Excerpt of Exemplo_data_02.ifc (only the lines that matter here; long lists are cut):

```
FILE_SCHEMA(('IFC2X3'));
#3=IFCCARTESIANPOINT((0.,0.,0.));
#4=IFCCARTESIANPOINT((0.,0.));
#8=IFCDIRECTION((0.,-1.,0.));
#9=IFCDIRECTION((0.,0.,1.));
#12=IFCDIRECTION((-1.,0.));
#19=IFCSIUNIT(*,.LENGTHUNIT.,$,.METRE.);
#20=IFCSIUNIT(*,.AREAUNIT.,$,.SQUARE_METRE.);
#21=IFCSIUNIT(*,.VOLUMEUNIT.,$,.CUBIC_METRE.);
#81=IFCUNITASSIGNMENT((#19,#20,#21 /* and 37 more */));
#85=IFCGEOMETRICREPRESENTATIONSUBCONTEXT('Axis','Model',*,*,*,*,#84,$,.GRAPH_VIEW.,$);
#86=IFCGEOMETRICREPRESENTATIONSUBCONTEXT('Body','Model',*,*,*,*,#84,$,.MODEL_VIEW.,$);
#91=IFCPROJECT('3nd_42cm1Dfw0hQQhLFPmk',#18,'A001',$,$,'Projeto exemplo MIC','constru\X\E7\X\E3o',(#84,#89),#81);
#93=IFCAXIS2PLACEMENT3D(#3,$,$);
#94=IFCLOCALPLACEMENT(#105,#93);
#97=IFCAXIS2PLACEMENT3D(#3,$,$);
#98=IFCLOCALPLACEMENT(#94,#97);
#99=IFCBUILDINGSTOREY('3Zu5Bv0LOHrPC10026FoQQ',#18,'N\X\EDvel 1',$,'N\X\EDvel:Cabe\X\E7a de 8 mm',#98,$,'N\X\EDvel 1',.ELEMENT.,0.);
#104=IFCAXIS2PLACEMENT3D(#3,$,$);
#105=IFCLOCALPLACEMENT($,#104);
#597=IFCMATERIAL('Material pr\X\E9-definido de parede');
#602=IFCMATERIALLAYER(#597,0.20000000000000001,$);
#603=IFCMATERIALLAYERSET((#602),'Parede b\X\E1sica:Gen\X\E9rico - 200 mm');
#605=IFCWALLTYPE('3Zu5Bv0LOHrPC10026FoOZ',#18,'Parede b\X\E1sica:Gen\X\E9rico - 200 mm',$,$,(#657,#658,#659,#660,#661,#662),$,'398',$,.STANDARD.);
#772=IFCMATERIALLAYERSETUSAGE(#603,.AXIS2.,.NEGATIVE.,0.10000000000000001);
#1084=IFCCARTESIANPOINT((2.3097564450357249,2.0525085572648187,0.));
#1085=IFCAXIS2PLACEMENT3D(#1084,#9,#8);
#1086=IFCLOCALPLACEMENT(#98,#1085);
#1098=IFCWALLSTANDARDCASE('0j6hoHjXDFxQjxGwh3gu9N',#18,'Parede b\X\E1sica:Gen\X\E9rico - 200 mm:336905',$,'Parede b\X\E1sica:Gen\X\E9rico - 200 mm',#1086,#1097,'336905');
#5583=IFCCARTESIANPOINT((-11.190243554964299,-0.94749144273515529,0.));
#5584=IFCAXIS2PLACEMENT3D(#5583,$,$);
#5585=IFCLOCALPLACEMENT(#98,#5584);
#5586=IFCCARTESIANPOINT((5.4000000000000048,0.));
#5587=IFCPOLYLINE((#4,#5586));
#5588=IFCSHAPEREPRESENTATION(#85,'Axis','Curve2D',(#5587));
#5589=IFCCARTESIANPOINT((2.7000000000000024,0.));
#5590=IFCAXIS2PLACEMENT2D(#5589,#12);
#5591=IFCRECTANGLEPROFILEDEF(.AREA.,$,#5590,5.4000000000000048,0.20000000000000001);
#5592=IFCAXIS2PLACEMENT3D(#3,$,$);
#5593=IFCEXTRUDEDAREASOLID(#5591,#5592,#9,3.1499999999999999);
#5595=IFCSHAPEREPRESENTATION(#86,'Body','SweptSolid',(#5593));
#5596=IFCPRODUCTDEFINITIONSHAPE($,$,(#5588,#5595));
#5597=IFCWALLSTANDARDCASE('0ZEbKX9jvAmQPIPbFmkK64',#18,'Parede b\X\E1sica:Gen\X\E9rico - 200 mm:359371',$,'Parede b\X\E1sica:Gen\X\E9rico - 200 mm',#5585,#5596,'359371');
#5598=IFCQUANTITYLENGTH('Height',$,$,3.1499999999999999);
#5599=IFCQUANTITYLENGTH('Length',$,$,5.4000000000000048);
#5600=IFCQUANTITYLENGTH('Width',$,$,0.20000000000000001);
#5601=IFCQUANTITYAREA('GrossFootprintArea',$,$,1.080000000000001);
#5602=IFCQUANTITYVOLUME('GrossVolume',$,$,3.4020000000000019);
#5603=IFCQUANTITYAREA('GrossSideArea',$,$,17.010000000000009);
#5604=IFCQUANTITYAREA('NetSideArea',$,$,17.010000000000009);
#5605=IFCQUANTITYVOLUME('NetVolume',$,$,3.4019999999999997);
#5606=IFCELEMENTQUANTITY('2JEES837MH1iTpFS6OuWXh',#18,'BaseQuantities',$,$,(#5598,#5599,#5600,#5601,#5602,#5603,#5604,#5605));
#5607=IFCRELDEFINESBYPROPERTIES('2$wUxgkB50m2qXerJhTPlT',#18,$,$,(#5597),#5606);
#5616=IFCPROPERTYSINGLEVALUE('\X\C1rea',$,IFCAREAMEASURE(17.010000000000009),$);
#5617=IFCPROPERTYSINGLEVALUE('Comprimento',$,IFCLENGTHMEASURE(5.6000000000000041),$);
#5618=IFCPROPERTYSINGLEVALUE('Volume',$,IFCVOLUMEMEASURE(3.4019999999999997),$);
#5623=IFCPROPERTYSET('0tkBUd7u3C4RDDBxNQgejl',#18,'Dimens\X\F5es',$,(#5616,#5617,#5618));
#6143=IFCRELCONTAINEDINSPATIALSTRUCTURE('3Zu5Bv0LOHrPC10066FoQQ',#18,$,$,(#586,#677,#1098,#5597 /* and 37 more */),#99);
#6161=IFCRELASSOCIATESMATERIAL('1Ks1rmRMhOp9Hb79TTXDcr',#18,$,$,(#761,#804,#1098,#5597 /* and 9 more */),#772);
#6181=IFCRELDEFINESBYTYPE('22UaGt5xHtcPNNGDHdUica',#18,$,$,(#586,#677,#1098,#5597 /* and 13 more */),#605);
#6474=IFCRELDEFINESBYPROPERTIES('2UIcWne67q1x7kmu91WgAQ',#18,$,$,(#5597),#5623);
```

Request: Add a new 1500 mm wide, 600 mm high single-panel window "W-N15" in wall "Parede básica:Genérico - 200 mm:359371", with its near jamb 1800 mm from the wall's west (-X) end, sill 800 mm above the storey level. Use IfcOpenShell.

```python
import numpy as np
import ifcopenshell
import ifcopenshell.api.feature
import ifcopenshell.api.geometry
import ifcopenshell.api.pset
import ifcopenshell.api.root
import ifcopenshell.api.spatial
import ifcopenshell.api.type
import ifcopenshell.geom
import ifcopenshell.util.element
import ifcopenshell.util.placement
import ifcopenshell.util.representation
import ifcopenshell.util.shape
import ifcopenshell.util.unit

model = ifcopenshell.open("Exemplo_data_02.ifc")
unit_scale = ifcopenshell.util.unit.calculate_unit_scale(model)
area_scale = ifcopenshell.util.unit.calculate_unit_scale(model, "AREAUNIT")
volume_scale = ifcopenshell.util.unit.calculate_unit_scale(model, "VOLUMEUNIT")
settings = ifcopenshell.geom.settings()


def volume(element):
    """Net volume in cubic metres, openings subtracted."""
    shape = ifcopenshell.geom.create_shape(settings, element)
    return ifcopenshell.util.shape.get_volume(shape.geometry)


wall = model.by_guid("0ZEbKX9jvAmQPIPbFmkK64")
storey = ifcopenshell.util.element.get_container(wall, ifc_class="IfcBuildingStorey")
context = ifcopenshell.util.representation.get_context(model, "Model", "Body", "MODEL_VIEW")
before = volume(wall)

width, height, from_end, sill = 1.5, 0.6, 1.8, 0.8  # metres

# The wall runs along its own X axis, and the end named is its -X end.
wall_shape = ifcopenshell.geom.create_shape(settings, wall)
x, y, z = ifcopenshell.util.shape.get_vertices(wall_shape.geometry).T
start = x.min() + from_end
face, thickness = float(y.min()), float(y.max() - y.min())
wall_matrix = ifcopenshell.util.placement.get_local_placement(wall.ObjectPlacement)
level = ifcopenshell.util.placement.get_local_placement(storey.ObjectPlacement)[2, 3]


def in_wall(x, y):
    """Placement at x, y metres in the wall's axes, at sill height."""
    matrix = wall_matrix.copy()
    matrix[:, 3] = wall_matrix @ np.array([x / unit_scale, y / unit_scale, 0.0, 1.0])
    matrix[2, 3] = level + sill / unit_scale
    return matrix


# Opening: a box that overshoots both wall faces by 50 mm.
opening = ifcopenshell.api.root.create_entity(model, ifc_class="IfcOpeningElement")
box = ifcopenshell.api.geometry.add_wall_representation(
    model, context=context, length=width, height=height, thickness=thickness + 0.1
)
ifcopenshell.api.geometry.assign_representation(model, product=opening, representation=box)
ifcopenshell.api.geometry.edit_object_placement(model, product=opening, matrix=in_wall(start, face - 0.05), is_si=False)
ifcopenshell.api.feature.add_feature(model, feature=opening, element=wall)

window = ifcopenshell.api.root.create_entity(model, ifc_class="IfcWindow", name="W-N15")
window.OverallWidth, window.OverallHeight = width / unit_scale, height / unit_scale
body = ifcopenshell.api.geometry.add_window_representation(
    model,
    context=context,
    overall_width=window.OverallWidth,
    overall_height=window.OverallHeight,
    partition_type="SINGLE_PANEL",
)
ifcopenshell.api.geometry.assign_representation(model, product=window, representation=body)
ifcopenshell.api.spatial.assign_container(model, products=[window], relating_structure=storey)
fills = ifcopenshell.api.feature.add_filling(model, opening=opening, element=window)
fills.OwnerHistory = window.OwnerHistory  # required in IFC2X3

# IFC2X3 keeps the operation on the window style.
style = ifcopenshell.api.root.create_entity(model, ifc_class="IfcWindowStyle", name="W-N15")
style.OperationType, style.ConstructionType = "SINGLE_PANEL", "NOTDEFINED"
style.ParameterTakesPrecedence = style.Sizeable = False
ifcopenshell.api.type.assign_type(model, related_objects=[window], relating_type=style)

# Centre the window in the wall's thickness.
ifcopenshell.api.geometry.edit_object_placement(model, product=window, matrix=in_wall(start, face), is_si=False)
window_shape = ifcopenshell.geom.create_shape(settings, window)
depth = ifcopenshell.util.shape.get_vertices(window_shape.geometry)[:, 1]
offset = face + thickness / 2 - (depth.min() + depth.max()) / 2
ifcopenshell.api.geometry.edit_object_placement(model, product=window, matrix=in_wall(start, offset), is_si=False)

after = volume(wall)

# Update the wall's stored quantities.
qto = model.by_id(ifcopenshell.util.element.get_pset(wall, "BaseQuantities", should_inherit=False)["id"])
ifcopenshell.api.pset.edit_qto(model, qto=qto, properties={
    "NetSideArea": after / thickness / area_scale,
    "NetVolume": after / volume_scale,
})
pset = model.by_id(ifcopenshell.util.element.get_pset(wall, "Dimensões", should_inherit=False)["id"])
ifcopenshell.api.pset.edit_pset(model, pset=pset, properties={
    "Área": model.create_entity("IfcAreaMeasure", after / thickness / area_scale),
    "Volume": model.create_entity("IfcVolumeMeasure", after / volume_scale),
})

print(f"wall volume {before:.3f} -> {after:.3f} m3")

model.write("Exemplo_data_02_v2.ifc")
```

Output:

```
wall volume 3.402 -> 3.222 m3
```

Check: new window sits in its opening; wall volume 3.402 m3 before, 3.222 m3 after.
